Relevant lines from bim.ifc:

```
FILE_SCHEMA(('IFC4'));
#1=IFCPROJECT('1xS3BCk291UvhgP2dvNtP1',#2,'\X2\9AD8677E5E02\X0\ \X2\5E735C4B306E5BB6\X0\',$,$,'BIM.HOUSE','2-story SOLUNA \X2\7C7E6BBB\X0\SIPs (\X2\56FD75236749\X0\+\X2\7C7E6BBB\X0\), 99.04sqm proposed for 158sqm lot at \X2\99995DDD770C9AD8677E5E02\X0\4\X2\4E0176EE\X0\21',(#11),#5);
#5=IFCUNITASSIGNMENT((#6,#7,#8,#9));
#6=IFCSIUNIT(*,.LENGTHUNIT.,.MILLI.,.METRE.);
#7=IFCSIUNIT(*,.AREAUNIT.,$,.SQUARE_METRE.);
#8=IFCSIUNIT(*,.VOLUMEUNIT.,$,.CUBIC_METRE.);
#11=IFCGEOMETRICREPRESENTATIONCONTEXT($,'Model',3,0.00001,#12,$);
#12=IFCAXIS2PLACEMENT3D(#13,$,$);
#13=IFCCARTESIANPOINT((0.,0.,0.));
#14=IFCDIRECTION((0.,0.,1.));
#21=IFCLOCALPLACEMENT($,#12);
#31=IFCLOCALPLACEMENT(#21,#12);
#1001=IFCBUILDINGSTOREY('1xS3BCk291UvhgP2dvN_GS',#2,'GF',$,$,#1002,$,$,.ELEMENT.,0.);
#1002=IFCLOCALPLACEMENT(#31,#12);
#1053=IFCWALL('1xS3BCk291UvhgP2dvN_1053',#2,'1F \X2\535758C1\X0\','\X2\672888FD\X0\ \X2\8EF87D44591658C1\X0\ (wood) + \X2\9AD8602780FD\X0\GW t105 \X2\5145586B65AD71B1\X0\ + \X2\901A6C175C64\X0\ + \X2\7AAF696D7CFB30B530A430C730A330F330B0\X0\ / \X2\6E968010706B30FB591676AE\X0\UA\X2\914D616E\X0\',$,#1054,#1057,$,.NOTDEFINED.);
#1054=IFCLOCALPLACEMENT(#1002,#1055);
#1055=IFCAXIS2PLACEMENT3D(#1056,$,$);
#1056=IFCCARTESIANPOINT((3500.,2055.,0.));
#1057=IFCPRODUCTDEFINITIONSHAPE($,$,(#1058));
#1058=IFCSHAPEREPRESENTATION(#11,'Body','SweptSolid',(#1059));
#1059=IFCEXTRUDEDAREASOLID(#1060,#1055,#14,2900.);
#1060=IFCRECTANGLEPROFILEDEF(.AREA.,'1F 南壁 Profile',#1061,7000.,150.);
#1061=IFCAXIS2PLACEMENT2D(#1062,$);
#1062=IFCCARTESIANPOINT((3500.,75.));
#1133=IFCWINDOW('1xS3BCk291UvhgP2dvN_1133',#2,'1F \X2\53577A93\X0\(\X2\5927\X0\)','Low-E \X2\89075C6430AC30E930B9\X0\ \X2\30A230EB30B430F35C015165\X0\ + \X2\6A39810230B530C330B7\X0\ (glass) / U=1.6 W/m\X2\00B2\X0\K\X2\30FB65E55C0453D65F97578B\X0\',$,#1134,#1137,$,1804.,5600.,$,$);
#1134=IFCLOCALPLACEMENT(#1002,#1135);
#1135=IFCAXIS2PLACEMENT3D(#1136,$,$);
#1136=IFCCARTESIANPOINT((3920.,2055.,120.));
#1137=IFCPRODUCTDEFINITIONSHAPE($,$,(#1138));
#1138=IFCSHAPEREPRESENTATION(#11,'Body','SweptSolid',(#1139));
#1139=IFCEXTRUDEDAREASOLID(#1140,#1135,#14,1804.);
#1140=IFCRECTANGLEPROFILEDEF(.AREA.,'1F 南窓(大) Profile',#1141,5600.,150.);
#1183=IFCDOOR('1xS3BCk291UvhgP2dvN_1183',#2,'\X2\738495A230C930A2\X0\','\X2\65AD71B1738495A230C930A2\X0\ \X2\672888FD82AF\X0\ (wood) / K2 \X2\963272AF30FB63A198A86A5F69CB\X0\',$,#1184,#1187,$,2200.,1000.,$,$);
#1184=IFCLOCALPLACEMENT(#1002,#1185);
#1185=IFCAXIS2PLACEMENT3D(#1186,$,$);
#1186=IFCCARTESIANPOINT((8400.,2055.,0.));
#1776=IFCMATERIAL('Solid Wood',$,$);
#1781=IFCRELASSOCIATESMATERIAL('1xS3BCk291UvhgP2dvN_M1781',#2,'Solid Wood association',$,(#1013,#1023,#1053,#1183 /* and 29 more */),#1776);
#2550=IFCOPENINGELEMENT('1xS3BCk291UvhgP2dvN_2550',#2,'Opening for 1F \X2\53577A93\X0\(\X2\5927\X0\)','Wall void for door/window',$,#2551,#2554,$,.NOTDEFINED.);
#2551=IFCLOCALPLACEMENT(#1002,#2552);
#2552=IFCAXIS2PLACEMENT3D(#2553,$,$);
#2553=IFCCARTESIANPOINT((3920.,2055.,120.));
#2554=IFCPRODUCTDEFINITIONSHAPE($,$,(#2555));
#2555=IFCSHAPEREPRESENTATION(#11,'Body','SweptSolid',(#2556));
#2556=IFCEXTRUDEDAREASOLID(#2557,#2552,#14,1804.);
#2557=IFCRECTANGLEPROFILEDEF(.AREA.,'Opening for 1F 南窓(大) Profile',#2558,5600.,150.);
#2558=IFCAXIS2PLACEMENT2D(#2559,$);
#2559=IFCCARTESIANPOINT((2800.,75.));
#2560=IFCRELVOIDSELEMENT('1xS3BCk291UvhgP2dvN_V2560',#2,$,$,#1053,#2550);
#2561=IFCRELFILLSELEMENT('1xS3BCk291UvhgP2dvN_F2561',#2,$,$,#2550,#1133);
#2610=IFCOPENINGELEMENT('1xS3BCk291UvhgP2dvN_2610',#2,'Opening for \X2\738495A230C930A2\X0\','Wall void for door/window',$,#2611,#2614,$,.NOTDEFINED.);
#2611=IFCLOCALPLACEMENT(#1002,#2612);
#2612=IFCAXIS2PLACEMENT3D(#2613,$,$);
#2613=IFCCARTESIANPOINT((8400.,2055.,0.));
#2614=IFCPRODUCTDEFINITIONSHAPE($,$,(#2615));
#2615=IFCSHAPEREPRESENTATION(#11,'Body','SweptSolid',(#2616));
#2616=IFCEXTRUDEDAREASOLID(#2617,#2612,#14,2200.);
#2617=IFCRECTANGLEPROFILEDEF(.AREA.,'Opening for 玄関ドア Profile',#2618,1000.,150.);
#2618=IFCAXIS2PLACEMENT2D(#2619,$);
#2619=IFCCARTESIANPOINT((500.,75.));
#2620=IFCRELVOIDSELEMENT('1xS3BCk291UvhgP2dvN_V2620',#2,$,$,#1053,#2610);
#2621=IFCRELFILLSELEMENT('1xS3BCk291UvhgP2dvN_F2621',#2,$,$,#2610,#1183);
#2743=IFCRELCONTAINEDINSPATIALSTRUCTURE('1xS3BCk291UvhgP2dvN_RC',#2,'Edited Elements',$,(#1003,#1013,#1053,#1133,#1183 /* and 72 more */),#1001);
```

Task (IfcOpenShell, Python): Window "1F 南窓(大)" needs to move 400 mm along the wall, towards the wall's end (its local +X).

```python
import ifcopenshell
import ifcopenshell.api.geometry
import ifcopenshell.util.placement

model = ifcopenshell.open("bim.ifc")

window = model.by_guid("1xS3BCk291UvhgP2dvN_1133")
opening = window.FillsVoids[0].RelatingOpeningElement
wall = opening.VoidsElements[0].RelatingBuildingElement

wall_matrix = ifcopenshell.util.placement.get_local_placement(wall.ObjectPlacement)
shift = wall_matrix[:3, 0] * 400.0
before = ifcopenshell.util.placement.get_local_placement(window.ObjectPlacement)[:3, 3].copy()

# The window is not placed relative to its opening, so move both.
for product in (opening, window):
    matrix = ifcopenshell.util.placement.get_local_placement(product.ObjectPlacement)
    matrix[:3, 3] += shift
    ifcopenshell.api.geometry.edit_object_placement(model, product=product, matrix=matrix, is_si=False)

after = ifcopenshell.util.placement.get_local_placement(window.ObjectPlacement)[:3, 3]
print("window moved by", (after - before).round(3) + 0.0)

model.write("bim_v2.ifc")
```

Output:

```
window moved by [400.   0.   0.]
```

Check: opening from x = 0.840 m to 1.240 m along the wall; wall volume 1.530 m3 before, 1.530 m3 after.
